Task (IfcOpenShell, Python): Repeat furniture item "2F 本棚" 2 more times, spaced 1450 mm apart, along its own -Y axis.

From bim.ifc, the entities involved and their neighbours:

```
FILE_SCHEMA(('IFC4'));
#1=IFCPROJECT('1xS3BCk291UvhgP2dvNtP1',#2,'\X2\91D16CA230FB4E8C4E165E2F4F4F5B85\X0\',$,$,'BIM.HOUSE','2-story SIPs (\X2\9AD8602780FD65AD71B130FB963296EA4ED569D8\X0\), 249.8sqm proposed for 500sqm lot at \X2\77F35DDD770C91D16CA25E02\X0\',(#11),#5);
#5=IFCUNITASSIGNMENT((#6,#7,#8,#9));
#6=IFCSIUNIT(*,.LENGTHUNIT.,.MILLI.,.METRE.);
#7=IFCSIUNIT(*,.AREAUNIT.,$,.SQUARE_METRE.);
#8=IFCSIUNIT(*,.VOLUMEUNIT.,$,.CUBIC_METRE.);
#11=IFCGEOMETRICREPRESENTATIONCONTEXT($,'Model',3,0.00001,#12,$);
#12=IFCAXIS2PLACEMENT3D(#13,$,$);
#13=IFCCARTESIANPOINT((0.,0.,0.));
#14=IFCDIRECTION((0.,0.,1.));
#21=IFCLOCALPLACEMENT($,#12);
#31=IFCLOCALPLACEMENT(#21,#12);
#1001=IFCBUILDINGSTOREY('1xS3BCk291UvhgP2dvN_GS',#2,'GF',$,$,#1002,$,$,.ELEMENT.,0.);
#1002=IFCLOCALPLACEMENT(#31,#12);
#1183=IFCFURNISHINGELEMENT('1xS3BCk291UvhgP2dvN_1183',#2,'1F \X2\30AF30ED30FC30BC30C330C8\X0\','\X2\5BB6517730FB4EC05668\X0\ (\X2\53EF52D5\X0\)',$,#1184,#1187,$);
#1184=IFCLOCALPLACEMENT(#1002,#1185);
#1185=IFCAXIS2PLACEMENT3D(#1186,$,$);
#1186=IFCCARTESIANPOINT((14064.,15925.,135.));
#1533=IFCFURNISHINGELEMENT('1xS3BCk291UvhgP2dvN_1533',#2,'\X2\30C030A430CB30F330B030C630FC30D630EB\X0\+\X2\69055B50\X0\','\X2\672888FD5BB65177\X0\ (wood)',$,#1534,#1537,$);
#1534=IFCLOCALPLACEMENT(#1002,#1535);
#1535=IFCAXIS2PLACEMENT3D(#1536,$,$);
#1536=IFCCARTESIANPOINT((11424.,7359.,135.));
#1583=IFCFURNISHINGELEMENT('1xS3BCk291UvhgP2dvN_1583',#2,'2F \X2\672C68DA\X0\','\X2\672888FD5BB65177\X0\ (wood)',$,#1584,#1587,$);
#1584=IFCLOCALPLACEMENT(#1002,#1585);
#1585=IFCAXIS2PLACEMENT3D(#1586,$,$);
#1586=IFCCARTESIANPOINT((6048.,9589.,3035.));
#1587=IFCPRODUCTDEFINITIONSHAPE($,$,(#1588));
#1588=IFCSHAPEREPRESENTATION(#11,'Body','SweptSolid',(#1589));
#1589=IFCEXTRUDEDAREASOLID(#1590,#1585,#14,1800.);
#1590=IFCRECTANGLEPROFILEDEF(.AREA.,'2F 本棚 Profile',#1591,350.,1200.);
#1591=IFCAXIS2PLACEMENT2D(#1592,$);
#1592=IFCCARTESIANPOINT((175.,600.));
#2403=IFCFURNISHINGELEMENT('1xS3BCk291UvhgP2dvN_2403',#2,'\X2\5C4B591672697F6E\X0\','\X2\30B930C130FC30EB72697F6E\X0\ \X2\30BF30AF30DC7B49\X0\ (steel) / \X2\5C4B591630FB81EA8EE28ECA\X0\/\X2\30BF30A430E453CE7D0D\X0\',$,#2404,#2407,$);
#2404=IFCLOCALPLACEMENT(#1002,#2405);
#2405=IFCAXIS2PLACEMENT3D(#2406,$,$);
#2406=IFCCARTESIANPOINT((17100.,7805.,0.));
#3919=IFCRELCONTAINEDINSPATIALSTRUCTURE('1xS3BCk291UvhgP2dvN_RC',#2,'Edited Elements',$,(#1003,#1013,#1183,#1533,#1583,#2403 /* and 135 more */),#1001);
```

```python
import ifcopenshell
import ifcopenshell.api.geometry
import ifcopenshell.api.root
import ifcopenshell.util.element
import ifcopenshell.util.placement

model = ifcopenshell.open("bim.ifc")


def reuse_history(source, copy):
    """copy_class also copies each property set's owner history, people and application; keep the originals."""
    for rel in copy.IsDefinedBy:
        if rel.is_a("IfcRelDefinesByProperties") and (history := rel.RelatingPropertyDefinition.OwnerHistory):
            rel.RelatingPropertyDefinition.OwnerHistory = source.OwnerHistory
            ifcopenshell.util.element.remove_deep2(model, history)


source = model.by_id(1583)
base = ifcopenshell.util.placement.get_local_placement(source.ObjectPlacement)
step = -base[:3, 1] * 1450.0

for i in range(1, 3):
    copy = ifcopenshell.api.root.copy_class(model, product=source)
    copy.Representation = ifcopenshell.util.element.copy_deep(
        model, source.Representation, exclude=["IfcGeometricRepresentationContext", "IfcRepresentationMap"]
    )
    reuse_history(source, copy)
    matrix = base.copy()
    matrix[:3, 3] += i * step
    print("added at", matrix[:3, 3].round(3) + 0.0)
    ifcopenshell.api.geometry.edit_object_placement(model, product=copy, matrix=matrix, is_si=False)

model.write("bim_updated.ifc")
```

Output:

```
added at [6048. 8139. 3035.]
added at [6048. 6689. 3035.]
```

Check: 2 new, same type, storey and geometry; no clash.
